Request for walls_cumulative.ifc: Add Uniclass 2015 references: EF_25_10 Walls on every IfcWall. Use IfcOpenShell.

First a look at what the model holds.

```python
import ifcopenshell

model = ifcopenshell.open("walls_cumulative.ifc")
print(model.schema)
print("classifications:", [c.Name for c in model.by_type("IfcClassification")])
for ifc_class in ("IfcDoor", "IfcRoof", "IfcStair", "IfcWall", "IfcWindow"):
    print(ifc_class, len(model.by_type(ifc_class)))
```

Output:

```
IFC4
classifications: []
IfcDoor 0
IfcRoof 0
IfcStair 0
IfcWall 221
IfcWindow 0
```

```python
import ifcopenshell
import ifcopenshell.api.classification

model = ifcopenshell.open("walls_cumulative.ifc")

system = ifcopenshell.api.classification.add_classification(model, classification="Uniclass 2015")

codes = {
    "IfcWall": ("EF_25_10", "Walls"),
}
for ifc_class, (code, name) in codes.items():
    products = model.by_type(ifc_class)
    ifcopenshell.api.classification.add_reference(
        model, products=products, classification=system, identification=code, name=name
    )
    print(code, len(products))

model.write("walls_cumulative_v2.ifc")
```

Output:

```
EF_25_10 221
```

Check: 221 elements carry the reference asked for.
